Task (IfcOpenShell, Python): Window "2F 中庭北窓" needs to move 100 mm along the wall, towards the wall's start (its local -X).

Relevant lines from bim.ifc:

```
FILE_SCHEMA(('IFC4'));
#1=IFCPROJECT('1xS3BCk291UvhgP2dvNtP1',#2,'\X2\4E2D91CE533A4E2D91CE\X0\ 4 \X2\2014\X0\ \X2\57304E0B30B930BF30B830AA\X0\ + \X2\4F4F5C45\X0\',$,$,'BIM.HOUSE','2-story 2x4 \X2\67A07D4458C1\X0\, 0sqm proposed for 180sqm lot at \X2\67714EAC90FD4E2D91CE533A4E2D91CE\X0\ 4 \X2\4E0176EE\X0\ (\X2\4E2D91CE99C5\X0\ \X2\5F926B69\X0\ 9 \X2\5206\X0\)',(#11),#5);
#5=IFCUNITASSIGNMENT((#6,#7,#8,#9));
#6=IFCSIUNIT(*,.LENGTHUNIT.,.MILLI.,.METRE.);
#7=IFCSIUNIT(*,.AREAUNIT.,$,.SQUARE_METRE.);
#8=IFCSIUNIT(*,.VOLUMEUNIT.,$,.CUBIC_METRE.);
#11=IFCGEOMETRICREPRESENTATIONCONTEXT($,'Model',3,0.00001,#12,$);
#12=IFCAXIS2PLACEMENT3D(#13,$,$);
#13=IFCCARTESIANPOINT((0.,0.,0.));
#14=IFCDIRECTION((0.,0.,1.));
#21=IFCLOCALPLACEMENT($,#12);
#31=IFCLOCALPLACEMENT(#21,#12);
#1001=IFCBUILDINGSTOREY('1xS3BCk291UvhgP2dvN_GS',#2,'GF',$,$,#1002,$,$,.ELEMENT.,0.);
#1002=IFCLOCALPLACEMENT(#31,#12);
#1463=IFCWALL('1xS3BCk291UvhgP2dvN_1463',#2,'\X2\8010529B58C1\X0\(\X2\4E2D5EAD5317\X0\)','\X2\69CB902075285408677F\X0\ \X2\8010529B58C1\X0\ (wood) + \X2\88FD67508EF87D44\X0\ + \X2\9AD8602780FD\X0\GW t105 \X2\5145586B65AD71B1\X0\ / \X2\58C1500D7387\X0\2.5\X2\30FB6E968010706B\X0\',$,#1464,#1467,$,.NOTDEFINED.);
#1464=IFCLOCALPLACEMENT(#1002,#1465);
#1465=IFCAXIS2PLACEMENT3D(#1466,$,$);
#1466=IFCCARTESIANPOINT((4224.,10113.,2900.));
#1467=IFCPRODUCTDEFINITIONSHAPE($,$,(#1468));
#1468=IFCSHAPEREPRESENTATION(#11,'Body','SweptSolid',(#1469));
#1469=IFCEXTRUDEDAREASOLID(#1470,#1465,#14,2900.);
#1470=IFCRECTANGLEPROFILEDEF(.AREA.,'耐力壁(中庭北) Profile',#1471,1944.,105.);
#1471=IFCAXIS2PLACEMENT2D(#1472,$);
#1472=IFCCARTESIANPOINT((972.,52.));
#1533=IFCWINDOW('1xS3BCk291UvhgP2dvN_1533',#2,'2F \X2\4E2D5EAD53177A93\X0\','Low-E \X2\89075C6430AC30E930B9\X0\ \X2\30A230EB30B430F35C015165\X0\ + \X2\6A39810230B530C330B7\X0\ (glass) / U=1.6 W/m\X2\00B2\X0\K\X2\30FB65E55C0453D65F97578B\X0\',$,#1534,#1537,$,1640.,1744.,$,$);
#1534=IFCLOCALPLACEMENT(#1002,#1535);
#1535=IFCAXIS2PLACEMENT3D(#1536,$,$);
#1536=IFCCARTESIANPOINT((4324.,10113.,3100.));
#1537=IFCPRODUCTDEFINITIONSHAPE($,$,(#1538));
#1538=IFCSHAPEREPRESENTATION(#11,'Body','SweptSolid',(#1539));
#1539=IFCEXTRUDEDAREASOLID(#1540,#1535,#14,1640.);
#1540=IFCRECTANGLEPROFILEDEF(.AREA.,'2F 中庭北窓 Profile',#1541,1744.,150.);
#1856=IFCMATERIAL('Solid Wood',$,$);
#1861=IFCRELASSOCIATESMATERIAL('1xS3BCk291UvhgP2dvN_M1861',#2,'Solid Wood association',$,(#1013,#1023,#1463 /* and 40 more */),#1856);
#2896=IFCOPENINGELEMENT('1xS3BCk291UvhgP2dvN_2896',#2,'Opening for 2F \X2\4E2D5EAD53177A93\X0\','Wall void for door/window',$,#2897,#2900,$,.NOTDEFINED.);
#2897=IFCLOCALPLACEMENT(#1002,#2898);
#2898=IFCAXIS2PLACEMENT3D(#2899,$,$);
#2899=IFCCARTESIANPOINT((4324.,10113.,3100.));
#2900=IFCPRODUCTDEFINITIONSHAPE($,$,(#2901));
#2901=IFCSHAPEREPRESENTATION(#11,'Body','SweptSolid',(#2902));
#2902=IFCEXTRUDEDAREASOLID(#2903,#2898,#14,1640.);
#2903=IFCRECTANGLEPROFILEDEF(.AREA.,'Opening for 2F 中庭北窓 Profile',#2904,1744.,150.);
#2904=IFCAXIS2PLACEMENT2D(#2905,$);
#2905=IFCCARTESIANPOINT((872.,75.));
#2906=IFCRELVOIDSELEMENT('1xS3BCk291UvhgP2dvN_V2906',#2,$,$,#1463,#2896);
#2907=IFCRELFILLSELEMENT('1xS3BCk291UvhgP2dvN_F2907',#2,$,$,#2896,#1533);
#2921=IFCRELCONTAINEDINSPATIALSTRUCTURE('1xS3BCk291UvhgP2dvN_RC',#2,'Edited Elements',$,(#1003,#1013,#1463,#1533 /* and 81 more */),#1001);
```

```python
import ifcopenshell
import ifcopenshell.api.geometry
import ifcopenshell.util.placement

model = ifcopenshell.open("bim.ifc")

window = model.by_guid("1xS3BCk291UvhgP2dvN_1533")
opening = window.FillsVoids[0].RelatingOpeningElement
wall = opening.VoidsElements[0].RelatingBuildingElement

wall_matrix = ifcopenshell.util.placement.get_local_placement(wall.ObjectPlacement)
shift = wall_matrix[:3, 0] * -100.0
before = ifcopenshell.util.placement.get_local_placement(window.ObjectPlacement)[:3, 3].copy()

# The window is not placed relative to its opening, so move both.
for product in (opening, window):
    matrix = ifcopenshell.util.placement.get_local_placement(product.ObjectPlacement)
    matrix[:3, 3] += shift
    ifcopenshell.api.geometry.edit_object_placement(model, product=product, matrix=matrix, is_si=False)

after = ifcopenshell.util.placement.get_local_placement(window.ObjectPlacement)[:3, 3]
print("window moved by", (after - before).round(3) + 0.0)

model.write("bim_rev.ifc")
```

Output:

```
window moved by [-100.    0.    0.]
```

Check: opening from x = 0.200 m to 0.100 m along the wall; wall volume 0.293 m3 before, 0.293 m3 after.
